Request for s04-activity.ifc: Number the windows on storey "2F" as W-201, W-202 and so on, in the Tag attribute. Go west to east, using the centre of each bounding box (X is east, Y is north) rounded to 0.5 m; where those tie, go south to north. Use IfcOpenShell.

First a look at what the model holds.

```python
import ifcopenshell
import ifcopenshell.util.element
import ifcopenshell.util.placement

model = ifcopenshell.open("s04-activity.ifc")
print(model.schema)
storey = next(s for s in model.by_type("IfcBuildingStorey") if s.Name == "2F")
windows = [e for e in ifcopenshell.util.element.get_decomposition(storey) if e.is_a("IfcWindow")]
for e in sorted(windows, key=lambda e: e.id()):
    origin = ifcopenshell.util.placement.get_local_placement(e.ObjectPlacement)[:3, 3]
    print(e.id(), e.Tag, e.Name, origin.round(2) + 0.0, sep=" | ")
```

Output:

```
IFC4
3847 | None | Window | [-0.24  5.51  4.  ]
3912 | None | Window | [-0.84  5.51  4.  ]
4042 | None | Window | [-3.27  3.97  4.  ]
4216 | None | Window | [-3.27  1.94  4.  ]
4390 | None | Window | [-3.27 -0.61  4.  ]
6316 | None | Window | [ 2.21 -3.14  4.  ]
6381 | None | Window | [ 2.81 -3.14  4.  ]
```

```python
import ifcopenshell
import ifcopenshell.geom
import ifcopenshell.util.element
import ifcopenshell.util.shape

model = ifcopenshell.open("s04-activity.ifc")
settings = ifcopenshell.geom.settings()
settings.set("use-world-coords", True)


def centre(element):
    shape = ifcopenshell.geom.create_shape(settings, element)
    return ifcopenshell.util.shape.get_bbox_centroid(shape.geometry)


storey = next(s for s in model.by_type("IfcBuildingStorey") if s.Name == "2F")
windows = [e for e in ifcopenshell.util.element.get_decomposition(storey) if e.is_a("IfcWindow")]

# Insertion points can sit at a corner or the storey origin, so sort by the geometry (in metres).
centres = {e: centre(e) for e in windows}
windows.sort(key=lambda e: (round(centres[e][0] / 0.5), centres[e][1]))

for i, e in enumerate(windows, start=1):
    number = f"W-2{i:02d}"
    e.Tag = number
    print(e.id(), number)

model.write("s04-activity_rev.ifc")
```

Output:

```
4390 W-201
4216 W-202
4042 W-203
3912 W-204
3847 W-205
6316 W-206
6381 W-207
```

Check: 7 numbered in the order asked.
